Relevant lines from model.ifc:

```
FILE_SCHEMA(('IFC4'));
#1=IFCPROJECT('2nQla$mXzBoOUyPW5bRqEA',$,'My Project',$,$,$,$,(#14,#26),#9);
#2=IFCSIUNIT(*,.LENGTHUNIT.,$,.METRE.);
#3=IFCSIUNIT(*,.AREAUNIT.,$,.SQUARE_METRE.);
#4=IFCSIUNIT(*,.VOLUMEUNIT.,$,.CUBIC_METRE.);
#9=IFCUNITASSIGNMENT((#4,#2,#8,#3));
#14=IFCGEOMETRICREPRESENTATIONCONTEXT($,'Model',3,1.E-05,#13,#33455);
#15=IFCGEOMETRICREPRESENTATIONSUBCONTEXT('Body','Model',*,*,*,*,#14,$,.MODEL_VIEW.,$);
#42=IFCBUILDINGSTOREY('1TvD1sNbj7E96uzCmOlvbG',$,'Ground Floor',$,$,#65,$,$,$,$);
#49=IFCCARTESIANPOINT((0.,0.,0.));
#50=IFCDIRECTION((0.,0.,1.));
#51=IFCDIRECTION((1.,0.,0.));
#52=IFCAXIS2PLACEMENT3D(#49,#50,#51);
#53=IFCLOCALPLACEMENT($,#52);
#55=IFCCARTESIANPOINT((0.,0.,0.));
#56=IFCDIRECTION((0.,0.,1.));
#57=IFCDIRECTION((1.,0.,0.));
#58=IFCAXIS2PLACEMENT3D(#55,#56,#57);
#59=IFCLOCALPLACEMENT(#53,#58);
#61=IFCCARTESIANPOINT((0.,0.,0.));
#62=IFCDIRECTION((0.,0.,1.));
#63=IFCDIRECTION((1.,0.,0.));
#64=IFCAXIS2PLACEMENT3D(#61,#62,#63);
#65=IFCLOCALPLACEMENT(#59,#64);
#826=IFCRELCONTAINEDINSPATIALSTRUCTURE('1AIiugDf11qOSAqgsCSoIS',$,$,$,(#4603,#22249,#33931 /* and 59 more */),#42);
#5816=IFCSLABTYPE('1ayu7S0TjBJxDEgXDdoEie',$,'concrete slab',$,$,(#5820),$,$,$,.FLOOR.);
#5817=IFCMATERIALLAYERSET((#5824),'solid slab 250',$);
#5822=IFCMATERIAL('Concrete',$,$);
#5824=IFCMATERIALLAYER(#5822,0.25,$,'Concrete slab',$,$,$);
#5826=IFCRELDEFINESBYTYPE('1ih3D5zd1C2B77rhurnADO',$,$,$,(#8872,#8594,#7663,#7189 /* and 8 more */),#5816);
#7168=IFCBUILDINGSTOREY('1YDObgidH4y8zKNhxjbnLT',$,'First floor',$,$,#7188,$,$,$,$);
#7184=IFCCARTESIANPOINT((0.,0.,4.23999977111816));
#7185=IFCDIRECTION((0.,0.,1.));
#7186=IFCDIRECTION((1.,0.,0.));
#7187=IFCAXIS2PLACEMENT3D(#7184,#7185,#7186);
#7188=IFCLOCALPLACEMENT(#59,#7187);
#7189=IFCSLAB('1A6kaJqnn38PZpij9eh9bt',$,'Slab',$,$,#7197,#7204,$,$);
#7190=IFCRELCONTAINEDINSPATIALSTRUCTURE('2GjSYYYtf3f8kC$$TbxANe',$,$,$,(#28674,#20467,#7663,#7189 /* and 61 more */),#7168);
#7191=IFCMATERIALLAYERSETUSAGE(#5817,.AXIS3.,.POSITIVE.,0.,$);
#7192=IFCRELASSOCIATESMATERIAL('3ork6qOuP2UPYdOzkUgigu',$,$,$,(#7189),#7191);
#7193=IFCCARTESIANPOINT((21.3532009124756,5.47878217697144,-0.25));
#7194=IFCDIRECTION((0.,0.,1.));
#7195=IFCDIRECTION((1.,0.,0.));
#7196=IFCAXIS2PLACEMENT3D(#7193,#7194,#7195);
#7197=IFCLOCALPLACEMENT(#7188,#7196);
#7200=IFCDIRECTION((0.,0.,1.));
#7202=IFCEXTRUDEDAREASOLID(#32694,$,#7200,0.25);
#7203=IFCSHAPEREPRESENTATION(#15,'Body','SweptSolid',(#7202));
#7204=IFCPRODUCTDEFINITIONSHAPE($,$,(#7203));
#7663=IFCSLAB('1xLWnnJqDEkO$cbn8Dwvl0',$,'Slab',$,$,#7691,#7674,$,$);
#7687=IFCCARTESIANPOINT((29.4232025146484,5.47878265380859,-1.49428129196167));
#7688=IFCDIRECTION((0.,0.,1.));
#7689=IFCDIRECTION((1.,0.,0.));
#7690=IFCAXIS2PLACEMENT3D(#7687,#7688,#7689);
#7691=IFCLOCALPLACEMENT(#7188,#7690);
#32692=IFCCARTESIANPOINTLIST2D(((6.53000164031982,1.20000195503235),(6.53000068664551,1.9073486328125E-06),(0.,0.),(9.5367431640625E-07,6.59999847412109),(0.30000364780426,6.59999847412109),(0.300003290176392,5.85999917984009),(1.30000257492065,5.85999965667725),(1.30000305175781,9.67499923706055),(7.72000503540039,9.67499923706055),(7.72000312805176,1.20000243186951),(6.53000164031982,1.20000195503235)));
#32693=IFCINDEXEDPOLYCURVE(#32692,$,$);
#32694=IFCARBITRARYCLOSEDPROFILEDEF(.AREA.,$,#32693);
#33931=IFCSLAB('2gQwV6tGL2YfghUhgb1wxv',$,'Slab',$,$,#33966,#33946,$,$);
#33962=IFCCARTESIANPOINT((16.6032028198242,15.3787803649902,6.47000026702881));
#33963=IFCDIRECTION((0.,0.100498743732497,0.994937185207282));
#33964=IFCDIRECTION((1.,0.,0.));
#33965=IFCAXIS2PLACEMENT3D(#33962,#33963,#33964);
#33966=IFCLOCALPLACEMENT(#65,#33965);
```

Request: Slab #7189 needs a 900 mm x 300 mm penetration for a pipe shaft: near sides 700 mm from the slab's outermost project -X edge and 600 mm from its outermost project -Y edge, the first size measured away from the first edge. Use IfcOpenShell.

```python
import numpy as np
import ifcopenshell
import ifcopenshell.api.feature
import ifcopenshell.api.geometry
import ifcopenshell.api.root
import ifcopenshell.geom
import ifcopenshell.util.placement
import ifcopenshell.util.representation
import ifcopenshell.util.shape
import ifcopenshell.util.unit

model = ifcopenshell.open("model.ifc")
unit_scale = ifcopenshell.util.unit.calculate_unit_scale(model)
settings = ifcopenshell.geom.settings()


def volume(element):
    """Net volume in cubic metres, openings subtracted."""
    shape = ifcopenshell.geom.create_shape(settings, element)
    return ifcopenshell.util.shape.get_volume(shape.geometry)


slab = model.by_id(7189)
before = volume(slab)

# Extent in the slab's own axes, in metres. The edges named are its -X and -Y sides.
slab_shape = ifcopenshell.geom.create_shape(settings, slab)
vertices = ifcopenshell.util.shape.get_vertices(slab_shape.geometry)
x_min, y_min, bottom = vertices.min(axis=0)
top = vertices[:, 2].max()

opening = ifcopenshell.api.root.create_entity(model, ifc_class="IfcOpeningElement", name="Pipe shaft opening", predefined_type="OPENING")
context = ifcopenshell.util.representation.get_context(model, "Model", "Body", "MODEL_VIEW")
width, depth = 0.9, 0.3
outline = [(0.0, 0.0), (width, 0.0), (width, depth), (0.0, depth), (0.0, 0.0)]
# Overshoot both faces by 50 mm so the cut is clean.
shape = ifcopenshell.api.geometry.add_slab_representation(
    model, context=context, depth=top - bottom + 0.1, polyline=outline
)
ifcopenshell.api.geometry.assign_representation(model, product=opening, representation=shape)

matrix = ifcopenshell.util.placement.get_local_placement(slab.ObjectPlacement)
matrix[:, 3] = matrix @ np.append(np.array([x_min + 0.7, y_min + 0.6, bottom - 0.05]) / unit_scale, 1.0)
ifcopenshell.api.geometry.edit_object_placement(model, product=opening, matrix=matrix, is_si=False)
ifcopenshell.api.feature.add_feature(model, feature=opening, element=slab)

after = volume(slab)

print(f"slab volume {before:.3f} -> {after:.3f} m3")

model.write("model_updated.ifc")
```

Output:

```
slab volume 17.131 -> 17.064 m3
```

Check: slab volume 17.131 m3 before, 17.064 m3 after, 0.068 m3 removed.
